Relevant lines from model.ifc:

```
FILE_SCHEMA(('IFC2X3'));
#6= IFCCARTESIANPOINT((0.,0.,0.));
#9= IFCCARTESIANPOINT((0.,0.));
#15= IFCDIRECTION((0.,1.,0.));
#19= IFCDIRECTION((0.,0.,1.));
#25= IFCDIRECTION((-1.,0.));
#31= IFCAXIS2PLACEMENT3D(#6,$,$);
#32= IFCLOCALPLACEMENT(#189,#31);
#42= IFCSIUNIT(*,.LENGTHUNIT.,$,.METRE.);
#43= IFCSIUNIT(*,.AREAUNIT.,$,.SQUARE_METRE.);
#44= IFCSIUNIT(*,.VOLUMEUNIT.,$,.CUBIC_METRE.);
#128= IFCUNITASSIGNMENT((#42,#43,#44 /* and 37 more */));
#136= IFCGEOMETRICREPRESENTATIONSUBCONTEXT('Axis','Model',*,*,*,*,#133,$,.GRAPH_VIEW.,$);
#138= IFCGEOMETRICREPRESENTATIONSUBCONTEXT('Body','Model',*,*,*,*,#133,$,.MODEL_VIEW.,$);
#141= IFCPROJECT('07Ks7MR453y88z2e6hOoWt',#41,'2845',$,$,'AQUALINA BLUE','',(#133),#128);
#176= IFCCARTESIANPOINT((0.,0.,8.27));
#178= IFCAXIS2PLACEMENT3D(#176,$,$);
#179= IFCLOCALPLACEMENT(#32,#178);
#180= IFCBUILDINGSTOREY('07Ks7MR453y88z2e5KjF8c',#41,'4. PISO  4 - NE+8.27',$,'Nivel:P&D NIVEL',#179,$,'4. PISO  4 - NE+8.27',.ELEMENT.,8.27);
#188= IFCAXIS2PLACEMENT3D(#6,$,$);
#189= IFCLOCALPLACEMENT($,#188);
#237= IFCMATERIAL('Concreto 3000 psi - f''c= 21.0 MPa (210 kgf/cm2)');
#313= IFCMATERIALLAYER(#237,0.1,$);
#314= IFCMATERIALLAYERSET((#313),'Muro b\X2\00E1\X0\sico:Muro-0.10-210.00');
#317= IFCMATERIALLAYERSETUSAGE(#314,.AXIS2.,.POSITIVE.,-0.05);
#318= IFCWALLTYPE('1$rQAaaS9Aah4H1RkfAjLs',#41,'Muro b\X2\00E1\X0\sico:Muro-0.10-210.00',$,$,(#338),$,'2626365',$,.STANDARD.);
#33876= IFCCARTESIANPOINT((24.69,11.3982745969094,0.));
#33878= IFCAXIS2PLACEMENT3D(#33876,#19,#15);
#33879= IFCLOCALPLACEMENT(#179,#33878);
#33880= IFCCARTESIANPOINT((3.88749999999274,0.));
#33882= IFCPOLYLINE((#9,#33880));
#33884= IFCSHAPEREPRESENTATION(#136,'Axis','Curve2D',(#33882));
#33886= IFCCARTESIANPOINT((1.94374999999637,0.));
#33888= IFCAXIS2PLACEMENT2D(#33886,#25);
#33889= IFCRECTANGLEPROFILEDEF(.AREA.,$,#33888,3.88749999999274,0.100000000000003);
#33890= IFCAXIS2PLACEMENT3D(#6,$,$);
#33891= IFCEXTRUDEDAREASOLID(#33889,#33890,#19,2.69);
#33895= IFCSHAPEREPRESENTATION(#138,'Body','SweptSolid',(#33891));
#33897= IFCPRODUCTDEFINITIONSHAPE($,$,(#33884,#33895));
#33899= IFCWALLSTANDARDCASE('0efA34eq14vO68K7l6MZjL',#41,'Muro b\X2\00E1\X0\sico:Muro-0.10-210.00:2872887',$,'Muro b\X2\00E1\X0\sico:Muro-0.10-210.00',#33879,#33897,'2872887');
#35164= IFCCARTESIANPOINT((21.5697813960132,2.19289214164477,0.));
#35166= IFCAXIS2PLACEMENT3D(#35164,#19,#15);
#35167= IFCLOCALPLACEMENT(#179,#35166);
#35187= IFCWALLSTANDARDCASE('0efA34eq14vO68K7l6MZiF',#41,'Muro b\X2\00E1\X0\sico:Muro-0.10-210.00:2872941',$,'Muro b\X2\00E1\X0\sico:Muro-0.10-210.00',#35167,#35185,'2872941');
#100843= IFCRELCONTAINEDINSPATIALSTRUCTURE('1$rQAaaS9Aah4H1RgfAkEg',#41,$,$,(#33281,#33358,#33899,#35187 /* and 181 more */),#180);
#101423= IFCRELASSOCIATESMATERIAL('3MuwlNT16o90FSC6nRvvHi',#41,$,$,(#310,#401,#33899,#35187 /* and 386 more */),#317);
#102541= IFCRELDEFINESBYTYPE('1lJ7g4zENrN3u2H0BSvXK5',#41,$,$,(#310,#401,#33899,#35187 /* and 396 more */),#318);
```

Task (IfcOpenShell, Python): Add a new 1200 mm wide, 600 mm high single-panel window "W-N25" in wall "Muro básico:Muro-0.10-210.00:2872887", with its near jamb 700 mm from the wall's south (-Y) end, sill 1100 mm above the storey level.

```python
import numpy as np
import ifcopenshell
import ifcopenshell.api.feature
import ifcopenshell.api.geometry
import ifcopenshell.api.root
import ifcopenshell.api.spatial
import ifcopenshell.api.type
import ifcopenshell.geom
import ifcopenshell.util.element
import ifcopenshell.util.placement
import ifcopenshell.util.representation
import ifcopenshell.util.shape
import ifcopenshell.util.unit

model = ifcopenshell.open("model.ifc")
unit_scale = ifcopenshell.util.unit.calculate_unit_scale(model)
settings = ifcopenshell.geom.settings()


def volume(element):
    """Net volume in cubic metres, openings subtracted."""
    shape = ifcopenshell.geom.create_shape(settings, element)
    return ifcopenshell.util.shape.get_volume(shape.geometry)


wall = model.by_guid("0efA34eq14vO68K7l6MZjL")
storey = ifcopenshell.util.element.get_container(wall, ifc_class="IfcBuildingStorey")
context = ifcopenshell.util.representation.get_context(model, "Model", "Body", "MODEL_VIEW")
before = volume(wall)

width, height, from_end, sill = 1.2, 0.6, 0.7, 1.1  # metres

# The wall runs along its own X axis, and the end named is its -X end.
wall_shape = ifcopenshell.geom.create_shape(settings, wall)
x, y, z = ifcopenshell.util.shape.get_vertices(wall_shape.geometry).T
start = x.min() + from_end
face, thickness = float(y.min()), float(y.max() - y.min())
wall_matrix = ifcopenshell.util.placement.get_local_placement(wall.ObjectPlacement)
level = ifcopenshell.util.placement.get_local_placement(storey.ObjectPlacement)[2, 3]


def in_wall(x, y):
    """Placement at x, y metres in the wall's axes, at sill height."""
    matrix = wall_matrix.copy()
    matrix[:, 3] = wall_matrix @ np.array([x / unit_scale, y / unit_scale, 0.0, 1.0])
    matrix[2, 3] = level + sill / unit_scale
    return matrix


# Opening: a box that overshoots both wall faces by 50 mm.
opening = ifcopenshell.api.root.create_entity(model, ifc_class="IfcOpeningElement")
box = ifcopenshell.api.geometry.add_wall_representation(
    model, context=context, length=width, height=height, thickness=thickness + 0.1
)
ifcopenshell.api.geometry.assign_representation(model, product=opening, representation=box)
ifcopenshell.api.geometry.edit_object_placement(model, product=opening, matrix=in_wall(start, face - 0.05), is_si=False)
ifcopenshell.api.feature.add_feature(model, feature=opening, element=wall)

window = ifcopenshell.api.root.create_entity(model, ifc_class="IfcWindow", name="W-N25")
window.OverallWidth, window.OverallHeight = width / unit_scale, height / unit_scale
body = ifcopenshell.api.geometry.add_window_representation(
    model,
    context=context,
    overall_width=window.OverallWidth,
    overall_height=window.OverallHeight,
    partition_type="SINGLE_PANEL",
)
ifcopenshell.api.geometry.assign_representation(model, product=window, representation=body)
ifcopenshell.api.spatial.assign_container(model, products=[window], relating_structure=storey)
fills = ifcopenshell.api.feature.add_filling(model, opening=opening, element=window)
fills.OwnerHistory = window.OwnerHistory  # required in IFC2X3

# IFC2X3 keeps the operation on the window style.
style = ifcopenshell.api.root.create_entity(model, ifc_class="IfcWindowStyle", name="W-N25")
style.OperationType, style.ConstructionType = "SINGLE_PANEL", "NOTDEFINED"
style.ParameterTakesPrecedence = style.Sizeable = False
ifcopenshell.api.type.assign_type(model, related_objects=[window], relating_type=style)

# Centre the window in the wall's thickness.
ifcopenshell.api.geometry.edit_object_placement(model, product=window, matrix=in_wall(start, face), is_si=False)
window_shape = ifcopenshell.geom.create_shape(settings, window)
depth = ifcopenshell.util.shape.get_vertices(window_shape.geometry)[:, 1]
offset = face + thickness / 2 - (depth.min() + depth.max()) / 2
ifcopenshell.api.geometry.edit_object_placement(model, product=window, matrix=in_wall(start, offset), is_si=False)

after = volume(wall)

print(f"wall volume {before:.3f} -> {after:.3f} m3")

model.write("model-out.ifc")
```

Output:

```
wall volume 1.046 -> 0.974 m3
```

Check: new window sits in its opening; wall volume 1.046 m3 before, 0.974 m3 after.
